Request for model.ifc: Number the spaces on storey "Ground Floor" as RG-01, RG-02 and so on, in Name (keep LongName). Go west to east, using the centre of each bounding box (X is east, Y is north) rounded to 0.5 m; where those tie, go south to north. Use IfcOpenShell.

First a look at what the model holds.

```python
import ifcopenshell
import ifcopenshell.util.element
import ifcopenshell.util.placement

model = ifcopenshell.open("model.ifc")
print(model.schema)
storey = next(s for s in model.by_type("IfcBuildingStorey") if s.Name == "Ground Floor")
spaces = [e for e in ifcopenshell.util.element.get_decomposition(storey) if e.is_a("IfcSpace")]
for e in sorted(spaces, key=lambda e: e.id()):
    origin = ifcopenshell.util.placement.get_local_placement(e.ObjectPlacement)[:3, 3]
    print(e.id(), e.Name, e.LongName, origin.round(2) + 0.0, sep=" | ")
```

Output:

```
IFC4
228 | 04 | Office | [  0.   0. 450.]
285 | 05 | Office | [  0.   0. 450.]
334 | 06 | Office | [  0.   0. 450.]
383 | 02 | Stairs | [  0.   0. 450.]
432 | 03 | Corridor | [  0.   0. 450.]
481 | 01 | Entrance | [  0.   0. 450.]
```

```python
import ifcopenshell
import ifcopenshell.geom
import ifcopenshell.util.element
import ifcopenshell.util.shape

model = ifcopenshell.open("model.ifc")
settings = ifcopenshell.geom.settings()
settings.set("use-world-coords", True)


def centre(element):
    shape = ifcopenshell.geom.create_shape(settings, element)
    return ifcopenshell.util.shape.get_bbox_centroid(shape.geometry)


storey = next(s for s in model.by_type("IfcBuildingStorey") if s.Name == "Ground Floor")
spaces = [e for e in ifcopenshell.util.element.get_decomposition(storey) if e.is_a("IfcSpace")]

# Insertion points can sit at a corner or the storey origin, so sort by the geometry (in metres).
centres = {e: centre(e) for e in spaces}
spaces.sort(key=lambda e: (round(centres[e][0] / 0.5), centres[e][1]))

for i, e in enumerate(spaces, start=1):
    number = f"RG-{i:02d}"
    e.Name = number
    print(e.id(), number)

model.write("model_v2.ifc")
```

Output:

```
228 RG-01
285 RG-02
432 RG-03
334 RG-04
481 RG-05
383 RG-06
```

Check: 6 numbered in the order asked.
